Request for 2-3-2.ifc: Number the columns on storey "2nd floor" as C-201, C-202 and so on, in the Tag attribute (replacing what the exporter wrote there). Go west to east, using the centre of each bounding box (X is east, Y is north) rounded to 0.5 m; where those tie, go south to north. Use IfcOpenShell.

First a look at what the model holds.

```python
import ifcopenshell
import ifcopenshell.util.element
import ifcopenshell.util.placement

model = ifcopenshell.open("2-3-2.ifc")
print(model.schema)
storey = next(s for s in model.by_type("IfcBuildingStorey") if s.Name == "2nd floor")
columns = [e for e in ifcopenshell.util.element.get_decomposition(storey) if e.is_a("IfcColumn")]
for e in sorted(columns, key=lambda e: e.id()):
    origin = ifcopenshell.util.placement.get_local_placement(e.ObjectPlacement)[:3, 3]
    print(e.id(), e.Tag, e.Name, origin.round(2) + 0.0, sep=" | ")
```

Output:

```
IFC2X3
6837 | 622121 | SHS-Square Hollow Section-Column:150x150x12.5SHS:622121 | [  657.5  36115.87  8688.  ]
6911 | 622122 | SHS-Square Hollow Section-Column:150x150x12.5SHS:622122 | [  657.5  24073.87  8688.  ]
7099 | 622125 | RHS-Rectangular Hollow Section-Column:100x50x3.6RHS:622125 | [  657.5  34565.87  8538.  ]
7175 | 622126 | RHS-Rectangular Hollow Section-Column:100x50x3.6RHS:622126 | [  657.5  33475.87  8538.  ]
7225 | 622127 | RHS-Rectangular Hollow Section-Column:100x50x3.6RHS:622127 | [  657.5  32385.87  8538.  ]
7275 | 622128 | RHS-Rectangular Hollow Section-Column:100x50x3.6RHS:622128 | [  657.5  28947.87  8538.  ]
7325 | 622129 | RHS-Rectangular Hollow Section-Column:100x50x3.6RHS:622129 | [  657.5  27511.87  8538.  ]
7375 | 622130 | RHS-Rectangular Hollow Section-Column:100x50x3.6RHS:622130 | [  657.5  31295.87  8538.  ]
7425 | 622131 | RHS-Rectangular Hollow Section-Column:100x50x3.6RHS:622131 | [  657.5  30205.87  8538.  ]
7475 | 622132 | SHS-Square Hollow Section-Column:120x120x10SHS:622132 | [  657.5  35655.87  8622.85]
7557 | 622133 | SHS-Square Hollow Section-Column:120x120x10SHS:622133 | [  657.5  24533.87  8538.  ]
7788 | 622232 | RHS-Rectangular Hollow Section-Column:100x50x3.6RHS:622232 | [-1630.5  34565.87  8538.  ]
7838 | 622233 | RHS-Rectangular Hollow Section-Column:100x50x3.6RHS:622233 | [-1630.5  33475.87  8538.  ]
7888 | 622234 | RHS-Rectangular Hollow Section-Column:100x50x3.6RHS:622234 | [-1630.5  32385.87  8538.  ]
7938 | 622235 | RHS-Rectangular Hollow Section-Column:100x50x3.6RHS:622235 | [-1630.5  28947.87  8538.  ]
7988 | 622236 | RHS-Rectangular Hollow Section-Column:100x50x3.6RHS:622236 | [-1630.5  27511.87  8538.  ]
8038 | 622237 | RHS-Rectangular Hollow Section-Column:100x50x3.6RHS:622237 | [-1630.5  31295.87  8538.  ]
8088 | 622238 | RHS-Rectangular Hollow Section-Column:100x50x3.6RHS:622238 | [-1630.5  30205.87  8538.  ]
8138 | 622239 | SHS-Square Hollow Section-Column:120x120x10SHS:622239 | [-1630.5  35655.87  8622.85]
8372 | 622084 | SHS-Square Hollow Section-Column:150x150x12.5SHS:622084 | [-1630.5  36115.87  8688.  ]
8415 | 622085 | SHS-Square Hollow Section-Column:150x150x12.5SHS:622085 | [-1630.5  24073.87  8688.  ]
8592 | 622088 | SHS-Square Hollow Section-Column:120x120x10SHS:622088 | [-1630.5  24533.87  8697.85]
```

```python
import ifcopenshell
import ifcopenshell.geom
import ifcopenshell.util.element
import ifcopenshell.util.shape

model = ifcopenshell.open("2-3-2.ifc")
settings = ifcopenshell.geom.settings()
settings.set("use-world-coords", True)


def centre(element):
    shape = ifcopenshell.geom.create_shape(settings, element)
    return ifcopenshell.util.shape.get_bbox_centroid(shape.geometry)


storey = next(s for s in model.by_type("IfcBuildingStorey") if s.Name == "2nd floor")
columns = [e for e in ifcopenshell.util.element.get_decomposition(storey) if e.is_a("IfcColumn")]

# Insertion points can sit at a corner or the storey origin, so sort by the geometry (in metres).
centres = {e: centre(e) for e in columns}
columns.sort(key=lambda e: (round(centres[e][0] / 0.5), centres[e][1]))

for i, e in enumerate(columns, start=1):
    number = f"C-2{i:02d}"
    e.Tag = number
    print(e.id(), number)

model.write("2-3-2_edited.ifc")
```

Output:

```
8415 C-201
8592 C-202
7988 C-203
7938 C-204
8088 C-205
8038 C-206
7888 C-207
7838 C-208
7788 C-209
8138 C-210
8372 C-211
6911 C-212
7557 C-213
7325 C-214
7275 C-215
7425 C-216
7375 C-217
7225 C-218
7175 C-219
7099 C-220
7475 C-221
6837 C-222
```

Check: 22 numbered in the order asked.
